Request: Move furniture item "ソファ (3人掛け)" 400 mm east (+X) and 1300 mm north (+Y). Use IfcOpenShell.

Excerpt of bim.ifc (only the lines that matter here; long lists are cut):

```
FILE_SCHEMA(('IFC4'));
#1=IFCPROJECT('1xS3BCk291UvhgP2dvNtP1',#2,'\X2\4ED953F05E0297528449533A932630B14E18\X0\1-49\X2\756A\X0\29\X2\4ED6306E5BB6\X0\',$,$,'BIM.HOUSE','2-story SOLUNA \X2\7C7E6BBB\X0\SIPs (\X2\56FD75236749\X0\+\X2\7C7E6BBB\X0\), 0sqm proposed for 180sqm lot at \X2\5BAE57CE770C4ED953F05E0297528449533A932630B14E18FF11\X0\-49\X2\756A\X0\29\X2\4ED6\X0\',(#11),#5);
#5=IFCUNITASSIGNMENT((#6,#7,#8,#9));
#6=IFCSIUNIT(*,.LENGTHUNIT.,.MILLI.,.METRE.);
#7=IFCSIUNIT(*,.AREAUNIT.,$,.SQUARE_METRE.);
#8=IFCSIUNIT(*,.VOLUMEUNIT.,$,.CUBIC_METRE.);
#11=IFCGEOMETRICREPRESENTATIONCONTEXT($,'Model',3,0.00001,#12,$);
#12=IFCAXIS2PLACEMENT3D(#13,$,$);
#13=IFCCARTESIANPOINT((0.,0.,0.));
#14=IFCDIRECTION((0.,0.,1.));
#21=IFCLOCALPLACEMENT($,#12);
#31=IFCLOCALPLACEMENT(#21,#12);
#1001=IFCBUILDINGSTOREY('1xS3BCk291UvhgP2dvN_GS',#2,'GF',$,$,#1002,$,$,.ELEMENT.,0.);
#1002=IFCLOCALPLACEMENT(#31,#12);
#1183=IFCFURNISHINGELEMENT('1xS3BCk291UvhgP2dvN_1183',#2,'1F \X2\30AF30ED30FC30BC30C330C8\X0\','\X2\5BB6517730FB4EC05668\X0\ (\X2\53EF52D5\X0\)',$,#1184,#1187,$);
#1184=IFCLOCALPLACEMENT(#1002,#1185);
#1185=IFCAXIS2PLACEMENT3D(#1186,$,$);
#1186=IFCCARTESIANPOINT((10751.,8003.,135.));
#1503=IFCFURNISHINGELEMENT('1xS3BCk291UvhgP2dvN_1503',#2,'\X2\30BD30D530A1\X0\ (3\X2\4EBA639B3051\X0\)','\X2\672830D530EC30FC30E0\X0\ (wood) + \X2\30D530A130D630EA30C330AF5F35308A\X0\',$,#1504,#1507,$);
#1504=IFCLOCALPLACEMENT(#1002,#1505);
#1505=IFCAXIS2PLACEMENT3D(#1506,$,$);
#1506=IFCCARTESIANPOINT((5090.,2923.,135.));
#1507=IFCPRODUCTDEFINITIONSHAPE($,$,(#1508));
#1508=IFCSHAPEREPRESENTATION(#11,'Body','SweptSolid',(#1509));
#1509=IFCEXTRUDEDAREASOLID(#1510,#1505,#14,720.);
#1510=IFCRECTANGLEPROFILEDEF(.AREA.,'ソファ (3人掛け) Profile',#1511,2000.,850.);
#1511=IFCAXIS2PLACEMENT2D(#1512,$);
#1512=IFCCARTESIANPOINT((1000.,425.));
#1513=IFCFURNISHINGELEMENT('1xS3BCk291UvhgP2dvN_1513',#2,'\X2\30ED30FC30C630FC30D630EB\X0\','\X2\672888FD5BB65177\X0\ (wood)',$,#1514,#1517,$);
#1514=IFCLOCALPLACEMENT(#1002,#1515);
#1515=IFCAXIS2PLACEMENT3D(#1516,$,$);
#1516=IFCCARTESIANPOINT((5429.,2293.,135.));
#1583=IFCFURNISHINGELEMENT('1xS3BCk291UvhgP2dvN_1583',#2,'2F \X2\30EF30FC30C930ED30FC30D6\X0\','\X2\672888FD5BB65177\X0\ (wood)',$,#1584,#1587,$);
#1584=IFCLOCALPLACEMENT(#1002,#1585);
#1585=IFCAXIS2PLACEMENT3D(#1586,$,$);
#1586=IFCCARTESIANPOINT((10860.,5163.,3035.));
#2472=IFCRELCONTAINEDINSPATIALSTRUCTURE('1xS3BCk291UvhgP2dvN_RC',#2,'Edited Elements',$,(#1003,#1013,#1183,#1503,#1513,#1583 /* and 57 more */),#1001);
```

```python
import ifcopenshell
import ifcopenshell.api.geometry
import ifcopenshell.util.placement
import ifcopenshell.util.unit

model = ifcopenshell.open("bim.ifc")
unit_scale = ifcopenshell.util.unit.calculate_unit_scale(model)

item = model.by_guid("1xS3BCk291UvhgP2dvN_1503")
matrix = ifcopenshell.util.placement.get_local_placement(item.ObjectPlacement)
matrix[0, 3] += 0.4 / unit_scale
matrix[1, 3] += 1.3 / unit_scale
ifcopenshell.api.geometry.edit_object_placement(model, product=item, matrix=matrix, is_si=False)

print(ifcopenshell.util.placement.get_local_placement(item.ObjectPlacement).round(3) + 0.0)

model.write("bim_rev.ifc")
```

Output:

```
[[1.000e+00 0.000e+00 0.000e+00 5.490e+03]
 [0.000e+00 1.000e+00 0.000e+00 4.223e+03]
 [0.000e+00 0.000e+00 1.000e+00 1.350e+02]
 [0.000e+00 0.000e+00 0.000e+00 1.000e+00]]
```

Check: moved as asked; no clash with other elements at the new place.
